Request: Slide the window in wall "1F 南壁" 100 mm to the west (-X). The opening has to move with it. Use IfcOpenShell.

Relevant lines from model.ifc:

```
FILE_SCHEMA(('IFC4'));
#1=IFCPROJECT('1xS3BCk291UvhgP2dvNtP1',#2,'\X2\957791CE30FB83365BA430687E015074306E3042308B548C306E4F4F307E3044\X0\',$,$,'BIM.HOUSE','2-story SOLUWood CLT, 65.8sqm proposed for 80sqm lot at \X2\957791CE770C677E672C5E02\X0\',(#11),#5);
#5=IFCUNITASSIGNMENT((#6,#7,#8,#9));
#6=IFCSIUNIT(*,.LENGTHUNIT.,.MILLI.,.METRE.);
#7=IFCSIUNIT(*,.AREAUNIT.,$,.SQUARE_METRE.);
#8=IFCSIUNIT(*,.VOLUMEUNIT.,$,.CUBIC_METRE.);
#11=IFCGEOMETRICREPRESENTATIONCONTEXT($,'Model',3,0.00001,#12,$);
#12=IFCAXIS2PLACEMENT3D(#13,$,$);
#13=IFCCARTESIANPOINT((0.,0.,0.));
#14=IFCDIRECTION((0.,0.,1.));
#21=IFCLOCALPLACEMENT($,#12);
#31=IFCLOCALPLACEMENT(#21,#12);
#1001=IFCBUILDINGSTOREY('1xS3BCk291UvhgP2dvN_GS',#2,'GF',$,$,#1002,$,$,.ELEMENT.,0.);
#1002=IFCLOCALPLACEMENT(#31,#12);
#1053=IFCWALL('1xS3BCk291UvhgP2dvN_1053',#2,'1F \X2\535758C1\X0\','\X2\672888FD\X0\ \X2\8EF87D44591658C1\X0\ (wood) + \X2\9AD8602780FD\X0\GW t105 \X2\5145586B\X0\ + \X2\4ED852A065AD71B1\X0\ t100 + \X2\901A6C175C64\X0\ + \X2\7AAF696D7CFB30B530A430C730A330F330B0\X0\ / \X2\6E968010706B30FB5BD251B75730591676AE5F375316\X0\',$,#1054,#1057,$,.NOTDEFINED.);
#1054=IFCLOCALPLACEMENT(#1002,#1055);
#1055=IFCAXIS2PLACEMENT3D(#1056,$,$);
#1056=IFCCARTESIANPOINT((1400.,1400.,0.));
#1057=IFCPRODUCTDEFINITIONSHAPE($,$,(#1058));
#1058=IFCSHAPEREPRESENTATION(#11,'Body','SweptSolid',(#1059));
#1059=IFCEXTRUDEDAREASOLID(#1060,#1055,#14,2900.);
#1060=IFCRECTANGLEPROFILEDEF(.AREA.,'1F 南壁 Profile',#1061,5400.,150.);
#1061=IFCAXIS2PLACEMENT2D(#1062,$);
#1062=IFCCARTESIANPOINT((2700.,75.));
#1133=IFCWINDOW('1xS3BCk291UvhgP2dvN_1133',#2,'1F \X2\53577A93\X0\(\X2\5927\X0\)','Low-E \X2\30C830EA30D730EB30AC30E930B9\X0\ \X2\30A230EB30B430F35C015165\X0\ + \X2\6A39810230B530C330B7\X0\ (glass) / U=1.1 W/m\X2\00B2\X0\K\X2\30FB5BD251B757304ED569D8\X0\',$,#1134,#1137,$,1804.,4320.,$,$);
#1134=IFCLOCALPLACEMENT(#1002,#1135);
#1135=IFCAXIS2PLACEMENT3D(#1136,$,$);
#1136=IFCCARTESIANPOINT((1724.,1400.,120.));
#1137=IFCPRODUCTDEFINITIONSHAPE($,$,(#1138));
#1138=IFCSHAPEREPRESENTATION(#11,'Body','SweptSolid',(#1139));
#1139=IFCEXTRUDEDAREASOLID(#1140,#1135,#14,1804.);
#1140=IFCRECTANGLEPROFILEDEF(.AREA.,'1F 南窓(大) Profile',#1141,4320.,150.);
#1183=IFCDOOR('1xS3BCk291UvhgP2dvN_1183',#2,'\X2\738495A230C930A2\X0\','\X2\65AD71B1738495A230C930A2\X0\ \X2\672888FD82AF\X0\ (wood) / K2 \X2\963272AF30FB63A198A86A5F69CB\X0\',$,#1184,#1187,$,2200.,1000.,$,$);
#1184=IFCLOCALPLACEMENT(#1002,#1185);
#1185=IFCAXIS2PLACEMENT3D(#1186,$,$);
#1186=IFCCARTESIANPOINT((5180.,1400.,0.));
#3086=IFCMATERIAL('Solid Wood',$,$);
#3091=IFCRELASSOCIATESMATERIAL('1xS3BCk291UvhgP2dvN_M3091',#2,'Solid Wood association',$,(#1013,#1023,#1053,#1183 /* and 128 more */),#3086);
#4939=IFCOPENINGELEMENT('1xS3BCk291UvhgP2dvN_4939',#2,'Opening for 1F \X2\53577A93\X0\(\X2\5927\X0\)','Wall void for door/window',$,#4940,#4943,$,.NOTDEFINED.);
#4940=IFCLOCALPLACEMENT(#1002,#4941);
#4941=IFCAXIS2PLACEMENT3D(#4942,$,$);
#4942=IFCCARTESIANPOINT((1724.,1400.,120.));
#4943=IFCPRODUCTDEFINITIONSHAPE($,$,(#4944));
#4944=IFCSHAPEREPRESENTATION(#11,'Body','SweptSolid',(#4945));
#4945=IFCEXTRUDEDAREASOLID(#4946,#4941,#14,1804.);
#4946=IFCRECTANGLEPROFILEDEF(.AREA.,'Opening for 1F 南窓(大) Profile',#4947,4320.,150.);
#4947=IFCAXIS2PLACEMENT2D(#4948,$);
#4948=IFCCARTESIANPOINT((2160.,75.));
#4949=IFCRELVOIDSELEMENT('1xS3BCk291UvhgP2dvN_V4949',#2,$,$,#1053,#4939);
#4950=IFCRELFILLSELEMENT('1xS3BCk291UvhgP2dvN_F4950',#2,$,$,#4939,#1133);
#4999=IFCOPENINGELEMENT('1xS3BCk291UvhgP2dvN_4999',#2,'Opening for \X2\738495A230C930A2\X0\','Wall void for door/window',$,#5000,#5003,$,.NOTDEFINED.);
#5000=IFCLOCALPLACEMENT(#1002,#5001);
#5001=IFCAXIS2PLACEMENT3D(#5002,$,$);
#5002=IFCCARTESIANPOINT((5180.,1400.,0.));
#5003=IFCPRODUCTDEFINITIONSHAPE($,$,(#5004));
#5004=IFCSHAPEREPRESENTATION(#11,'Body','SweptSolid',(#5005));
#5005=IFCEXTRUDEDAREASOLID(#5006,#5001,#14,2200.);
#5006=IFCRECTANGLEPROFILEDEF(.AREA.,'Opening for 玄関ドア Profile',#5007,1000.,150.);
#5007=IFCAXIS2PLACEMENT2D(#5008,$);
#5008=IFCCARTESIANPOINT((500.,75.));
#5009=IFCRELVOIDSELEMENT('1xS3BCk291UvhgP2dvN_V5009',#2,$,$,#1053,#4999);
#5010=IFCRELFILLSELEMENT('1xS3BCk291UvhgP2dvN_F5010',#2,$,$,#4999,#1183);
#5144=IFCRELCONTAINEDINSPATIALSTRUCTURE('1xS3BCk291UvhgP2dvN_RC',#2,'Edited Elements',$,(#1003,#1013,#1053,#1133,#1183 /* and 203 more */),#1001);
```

```python
import ifcopenshell
import ifcopenshell.api.geometry
import ifcopenshell.util.placement

model = ifcopenshell.open("model.ifc")

window = model.by_guid("1xS3BCk291UvhgP2dvN_1133")
opening = window.FillsVoids[0].RelatingOpeningElement
wall = opening.VoidsElements[0].RelatingBuildingElement

wall_matrix = ifcopenshell.util.placement.get_local_placement(wall.ObjectPlacement)
shift = wall_matrix[:3, 0] * -100.0
before = ifcopenshell.util.placement.get_local_placement(window.ObjectPlacement)[:3, 3].copy()

# The window is not placed relative to its opening, so move both.
for product in (opening, window):
    matrix = ifcopenshell.util.placement.get_local_placement(product.ObjectPlacement)
    matrix[:3, 3] += shift
    ifcopenshell.api.geometry.edit_object_placement(model, product=product, matrix=matrix, is_si=False)

after = ifcopenshell.util.placement.get_local_placement(window.ObjectPlacement)[:3, 3]
print("window moved by", (after - before).round(3) + 0.0)

model.write("model_v2.ifc")
```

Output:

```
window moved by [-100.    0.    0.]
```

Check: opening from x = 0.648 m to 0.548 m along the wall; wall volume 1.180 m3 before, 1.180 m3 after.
